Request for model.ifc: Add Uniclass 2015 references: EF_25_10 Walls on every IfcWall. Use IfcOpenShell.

First a look at what the model holds.

```python
import ifcopenshell

model = ifcopenshell.open("model.ifc")
print(model.schema)
print("classifications:", [c.Name for c in model.by_type("IfcClassification")])
for ifc_class in ("IfcDoor", "IfcRoof", "IfcStair", "IfcWall", "IfcWindow"):
    print(ifc_class, len(model.by_type(ifc_class)))
```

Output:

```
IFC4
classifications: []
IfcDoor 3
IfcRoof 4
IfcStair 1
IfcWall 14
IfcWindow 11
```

```python
import ifcopenshell
import ifcopenshell.api.classification

model = ifcopenshell.open("model.ifc")

system = ifcopenshell.api.classification.add_classification(model, classification="Uniclass 2015")

codes = {
    "IfcWall": ("EF_25_10", "Walls"),
}
for ifc_class, (code, name) in codes.items():
    products = model.by_type(ifc_class)
    ifcopenshell.api.classification.add_reference(
        model, products=products, classification=system, identification=code, name=name
    )
    print(code, len(products))

model.write("model_rev.ifc")
```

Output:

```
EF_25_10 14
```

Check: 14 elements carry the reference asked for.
